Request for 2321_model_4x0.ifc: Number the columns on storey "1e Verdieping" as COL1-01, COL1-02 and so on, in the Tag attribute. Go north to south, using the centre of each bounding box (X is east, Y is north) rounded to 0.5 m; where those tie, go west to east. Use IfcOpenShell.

First a look at what the model holds.

```python
import ifcopenshell
import ifcopenshell.util.element
import ifcopenshell.util.placement

model = ifcopenshell.open("2321_model_4x0.ifc")
print(model.schema)
storey = next(s for s in model.by_type("IfcBuildingStorey") if s.Name == "1e Verdieping")
columns = [e for e in ifcopenshell.util.element.get_decomposition(storey) if e.is_a("IfcColumn")]
for e in sorted(columns, key=lambda e: e.id()):
    origin = ifcopenshell.util.placement.get_local_placement(e.ObjectPlacement)[:3, 3]
    print(e.id(), e.Tag, e.Name, origin.round(2) + 0.0, sep=" | ")
```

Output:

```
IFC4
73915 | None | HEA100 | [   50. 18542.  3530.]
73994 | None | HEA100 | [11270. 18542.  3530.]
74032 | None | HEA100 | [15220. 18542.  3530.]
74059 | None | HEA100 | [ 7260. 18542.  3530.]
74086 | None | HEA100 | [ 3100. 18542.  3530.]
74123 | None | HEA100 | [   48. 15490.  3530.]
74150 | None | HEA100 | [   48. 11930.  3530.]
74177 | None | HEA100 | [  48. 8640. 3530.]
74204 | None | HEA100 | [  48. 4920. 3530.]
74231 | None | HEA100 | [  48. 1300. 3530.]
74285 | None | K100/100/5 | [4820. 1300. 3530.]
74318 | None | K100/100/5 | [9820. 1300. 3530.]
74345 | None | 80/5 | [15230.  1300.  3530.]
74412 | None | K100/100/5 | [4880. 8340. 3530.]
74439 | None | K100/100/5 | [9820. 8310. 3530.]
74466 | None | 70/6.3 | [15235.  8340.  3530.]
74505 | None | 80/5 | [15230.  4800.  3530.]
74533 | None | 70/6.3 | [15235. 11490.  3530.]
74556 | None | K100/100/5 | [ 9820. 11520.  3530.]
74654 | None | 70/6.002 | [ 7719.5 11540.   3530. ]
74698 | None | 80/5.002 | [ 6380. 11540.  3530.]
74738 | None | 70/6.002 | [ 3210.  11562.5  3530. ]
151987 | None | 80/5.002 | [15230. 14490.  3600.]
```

```python
import ifcopenshell
import ifcopenshell.geom
import ifcopenshell.util.element
import ifcopenshell.util.shape

model = ifcopenshell.open("2321_model_4x0.ifc")
settings = ifcopenshell.geom.settings()
settings.set("use-world-coords", True)


def centre(element):
    shape = ifcopenshell.geom.create_shape(settings, element)
    return ifcopenshell.util.shape.get_bbox_centroid(shape.geometry)


storey = next(s for s in model.by_type("IfcBuildingStorey") if s.Name == "1e Verdieping")
columns = [e for e in ifcopenshell.util.element.get_decomposition(storey) if e.is_a("IfcColumn")]

# Insertion points can sit at a corner or the storey origin, so sort by the geometry (in metres).
centres = {e: centre(e) for e in columns}
columns.sort(key=lambda e: (-round(centres[e][1] / 0.5), centres[e][0]))

for i, e in enumerate(columns, start=1):
    number = f"COL1-{i:02d}"
    e.Tag = number
    print(e.id(), number)

model.write("2321_model_4x0_updated.ifc")
```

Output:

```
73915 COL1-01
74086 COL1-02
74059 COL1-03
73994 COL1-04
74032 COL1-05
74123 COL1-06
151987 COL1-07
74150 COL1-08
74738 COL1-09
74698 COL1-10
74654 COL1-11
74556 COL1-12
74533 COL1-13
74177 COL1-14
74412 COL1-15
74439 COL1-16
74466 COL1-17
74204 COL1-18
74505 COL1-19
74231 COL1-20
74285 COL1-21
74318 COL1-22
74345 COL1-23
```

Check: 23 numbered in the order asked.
